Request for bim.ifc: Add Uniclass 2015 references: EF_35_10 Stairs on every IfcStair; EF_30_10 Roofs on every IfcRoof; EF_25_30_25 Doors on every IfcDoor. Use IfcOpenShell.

First a look at what the model holds.

```python
import ifcopenshell

model = ifcopenshell.open("bim.ifc")
print(model.schema)
print("classifications:", [c.Name for c in model.by_type("IfcClassification")])
for ifc_class in ("IfcDoor", "IfcRoof", "IfcStair", "IfcWall", "IfcWindow"):
    print(ifc_class, len(model.by_type(ifc_class)))
```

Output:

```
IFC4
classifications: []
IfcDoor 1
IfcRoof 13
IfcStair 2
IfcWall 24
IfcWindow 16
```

```python
import ifcopenshell
import ifcopenshell.api.classification

model = ifcopenshell.open("bim.ifc")

system = ifcopenshell.api.classification.add_classification(model, classification="Uniclass 2015")

codes = {
    "IfcStair": ("EF_35_10", "Stairs"),
    "IfcRoof": ("EF_30_10", "Roofs"),
    "IfcDoor": ("EF_25_30_25", "Doors"),
}
for ifc_class, (code, name) in codes.items():
    products = model.by_type(ifc_class)
    ifcopenshell.api.classification.add_reference(
        model, products=products, classification=system, identification=code, name=name
    )
    print(code, len(products))

model.write("bim-out.ifc")
```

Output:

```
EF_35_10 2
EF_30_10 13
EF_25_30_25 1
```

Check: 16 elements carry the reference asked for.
